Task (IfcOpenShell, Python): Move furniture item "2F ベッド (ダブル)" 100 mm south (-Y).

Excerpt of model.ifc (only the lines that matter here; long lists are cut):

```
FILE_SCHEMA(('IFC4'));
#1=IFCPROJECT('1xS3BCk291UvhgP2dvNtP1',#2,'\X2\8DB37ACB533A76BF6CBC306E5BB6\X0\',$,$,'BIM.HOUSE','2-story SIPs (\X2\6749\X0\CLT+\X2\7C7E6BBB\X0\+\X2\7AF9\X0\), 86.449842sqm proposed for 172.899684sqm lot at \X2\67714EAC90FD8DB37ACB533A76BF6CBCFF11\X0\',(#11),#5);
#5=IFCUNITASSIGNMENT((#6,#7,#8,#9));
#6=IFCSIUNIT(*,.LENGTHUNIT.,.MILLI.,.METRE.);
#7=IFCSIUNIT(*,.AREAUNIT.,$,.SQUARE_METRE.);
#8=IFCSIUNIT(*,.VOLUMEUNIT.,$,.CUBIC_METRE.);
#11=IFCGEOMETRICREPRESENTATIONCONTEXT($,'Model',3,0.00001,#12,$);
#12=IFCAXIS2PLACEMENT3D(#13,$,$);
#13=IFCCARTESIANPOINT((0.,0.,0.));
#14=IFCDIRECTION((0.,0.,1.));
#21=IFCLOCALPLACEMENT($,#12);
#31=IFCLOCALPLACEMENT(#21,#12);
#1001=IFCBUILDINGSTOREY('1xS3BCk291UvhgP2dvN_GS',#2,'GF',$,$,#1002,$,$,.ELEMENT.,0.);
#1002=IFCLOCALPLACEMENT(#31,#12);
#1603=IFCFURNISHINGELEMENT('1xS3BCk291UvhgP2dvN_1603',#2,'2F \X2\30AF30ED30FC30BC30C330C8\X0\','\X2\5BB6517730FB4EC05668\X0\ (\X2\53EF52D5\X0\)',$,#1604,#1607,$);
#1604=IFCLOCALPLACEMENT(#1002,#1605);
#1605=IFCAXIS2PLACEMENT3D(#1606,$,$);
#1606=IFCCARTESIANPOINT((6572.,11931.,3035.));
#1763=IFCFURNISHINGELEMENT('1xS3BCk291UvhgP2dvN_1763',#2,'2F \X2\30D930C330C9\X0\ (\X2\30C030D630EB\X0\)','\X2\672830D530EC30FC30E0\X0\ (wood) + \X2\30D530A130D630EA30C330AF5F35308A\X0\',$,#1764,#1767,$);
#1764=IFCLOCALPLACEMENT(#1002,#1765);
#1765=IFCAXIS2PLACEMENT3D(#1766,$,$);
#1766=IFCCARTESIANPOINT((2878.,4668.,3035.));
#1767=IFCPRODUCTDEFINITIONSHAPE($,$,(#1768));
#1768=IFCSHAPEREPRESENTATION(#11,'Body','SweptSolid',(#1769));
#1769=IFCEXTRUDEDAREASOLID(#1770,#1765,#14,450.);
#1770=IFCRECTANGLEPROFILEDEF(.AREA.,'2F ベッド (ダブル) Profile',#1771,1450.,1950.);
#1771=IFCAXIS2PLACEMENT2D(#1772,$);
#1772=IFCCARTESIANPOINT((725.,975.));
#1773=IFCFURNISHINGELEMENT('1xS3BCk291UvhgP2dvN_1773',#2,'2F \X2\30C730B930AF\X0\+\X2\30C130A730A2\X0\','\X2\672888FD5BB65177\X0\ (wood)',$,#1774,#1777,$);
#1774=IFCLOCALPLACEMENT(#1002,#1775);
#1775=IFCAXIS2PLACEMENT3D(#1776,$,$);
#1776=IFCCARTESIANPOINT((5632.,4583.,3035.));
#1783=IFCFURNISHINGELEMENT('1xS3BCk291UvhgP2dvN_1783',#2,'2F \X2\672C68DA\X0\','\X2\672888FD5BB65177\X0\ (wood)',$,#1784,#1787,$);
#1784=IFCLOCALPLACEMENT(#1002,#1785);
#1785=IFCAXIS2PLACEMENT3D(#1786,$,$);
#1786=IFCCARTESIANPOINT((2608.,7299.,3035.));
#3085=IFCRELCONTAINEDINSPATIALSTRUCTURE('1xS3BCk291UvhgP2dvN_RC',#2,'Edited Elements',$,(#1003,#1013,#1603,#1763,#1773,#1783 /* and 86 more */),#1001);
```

```python
import ifcopenshell
import ifcopenshell.api.geometry
import ifcopenshell.util.placement
import ifcopenshell.util.unit

model = ifcopenshell.open("model.ifc")
unit_scale = ifcopenshell.util.unit.calculate_unit_scale(model)

item = model.by_guid("1xS3BCk291UvhgP2dvN_1763")
matrix = ifcopenshell.util.placement.get_local_placement(item.ObjectPlacement)
matrix[1, 3] -= 0.1 / unit_scale
ifcopenshell.api.geometry.edit_object_placement(model, product=item, matrix=matrix, is_si=False)

print(ifcopenshell.util.placement.get_local_placement(item.ObjectPlacement).round(3) + 0.0)

model.write("model_v2.ifc")
```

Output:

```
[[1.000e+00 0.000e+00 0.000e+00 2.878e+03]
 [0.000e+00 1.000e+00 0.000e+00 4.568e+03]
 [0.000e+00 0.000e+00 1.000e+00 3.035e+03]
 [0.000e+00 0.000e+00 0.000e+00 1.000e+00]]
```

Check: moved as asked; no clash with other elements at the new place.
